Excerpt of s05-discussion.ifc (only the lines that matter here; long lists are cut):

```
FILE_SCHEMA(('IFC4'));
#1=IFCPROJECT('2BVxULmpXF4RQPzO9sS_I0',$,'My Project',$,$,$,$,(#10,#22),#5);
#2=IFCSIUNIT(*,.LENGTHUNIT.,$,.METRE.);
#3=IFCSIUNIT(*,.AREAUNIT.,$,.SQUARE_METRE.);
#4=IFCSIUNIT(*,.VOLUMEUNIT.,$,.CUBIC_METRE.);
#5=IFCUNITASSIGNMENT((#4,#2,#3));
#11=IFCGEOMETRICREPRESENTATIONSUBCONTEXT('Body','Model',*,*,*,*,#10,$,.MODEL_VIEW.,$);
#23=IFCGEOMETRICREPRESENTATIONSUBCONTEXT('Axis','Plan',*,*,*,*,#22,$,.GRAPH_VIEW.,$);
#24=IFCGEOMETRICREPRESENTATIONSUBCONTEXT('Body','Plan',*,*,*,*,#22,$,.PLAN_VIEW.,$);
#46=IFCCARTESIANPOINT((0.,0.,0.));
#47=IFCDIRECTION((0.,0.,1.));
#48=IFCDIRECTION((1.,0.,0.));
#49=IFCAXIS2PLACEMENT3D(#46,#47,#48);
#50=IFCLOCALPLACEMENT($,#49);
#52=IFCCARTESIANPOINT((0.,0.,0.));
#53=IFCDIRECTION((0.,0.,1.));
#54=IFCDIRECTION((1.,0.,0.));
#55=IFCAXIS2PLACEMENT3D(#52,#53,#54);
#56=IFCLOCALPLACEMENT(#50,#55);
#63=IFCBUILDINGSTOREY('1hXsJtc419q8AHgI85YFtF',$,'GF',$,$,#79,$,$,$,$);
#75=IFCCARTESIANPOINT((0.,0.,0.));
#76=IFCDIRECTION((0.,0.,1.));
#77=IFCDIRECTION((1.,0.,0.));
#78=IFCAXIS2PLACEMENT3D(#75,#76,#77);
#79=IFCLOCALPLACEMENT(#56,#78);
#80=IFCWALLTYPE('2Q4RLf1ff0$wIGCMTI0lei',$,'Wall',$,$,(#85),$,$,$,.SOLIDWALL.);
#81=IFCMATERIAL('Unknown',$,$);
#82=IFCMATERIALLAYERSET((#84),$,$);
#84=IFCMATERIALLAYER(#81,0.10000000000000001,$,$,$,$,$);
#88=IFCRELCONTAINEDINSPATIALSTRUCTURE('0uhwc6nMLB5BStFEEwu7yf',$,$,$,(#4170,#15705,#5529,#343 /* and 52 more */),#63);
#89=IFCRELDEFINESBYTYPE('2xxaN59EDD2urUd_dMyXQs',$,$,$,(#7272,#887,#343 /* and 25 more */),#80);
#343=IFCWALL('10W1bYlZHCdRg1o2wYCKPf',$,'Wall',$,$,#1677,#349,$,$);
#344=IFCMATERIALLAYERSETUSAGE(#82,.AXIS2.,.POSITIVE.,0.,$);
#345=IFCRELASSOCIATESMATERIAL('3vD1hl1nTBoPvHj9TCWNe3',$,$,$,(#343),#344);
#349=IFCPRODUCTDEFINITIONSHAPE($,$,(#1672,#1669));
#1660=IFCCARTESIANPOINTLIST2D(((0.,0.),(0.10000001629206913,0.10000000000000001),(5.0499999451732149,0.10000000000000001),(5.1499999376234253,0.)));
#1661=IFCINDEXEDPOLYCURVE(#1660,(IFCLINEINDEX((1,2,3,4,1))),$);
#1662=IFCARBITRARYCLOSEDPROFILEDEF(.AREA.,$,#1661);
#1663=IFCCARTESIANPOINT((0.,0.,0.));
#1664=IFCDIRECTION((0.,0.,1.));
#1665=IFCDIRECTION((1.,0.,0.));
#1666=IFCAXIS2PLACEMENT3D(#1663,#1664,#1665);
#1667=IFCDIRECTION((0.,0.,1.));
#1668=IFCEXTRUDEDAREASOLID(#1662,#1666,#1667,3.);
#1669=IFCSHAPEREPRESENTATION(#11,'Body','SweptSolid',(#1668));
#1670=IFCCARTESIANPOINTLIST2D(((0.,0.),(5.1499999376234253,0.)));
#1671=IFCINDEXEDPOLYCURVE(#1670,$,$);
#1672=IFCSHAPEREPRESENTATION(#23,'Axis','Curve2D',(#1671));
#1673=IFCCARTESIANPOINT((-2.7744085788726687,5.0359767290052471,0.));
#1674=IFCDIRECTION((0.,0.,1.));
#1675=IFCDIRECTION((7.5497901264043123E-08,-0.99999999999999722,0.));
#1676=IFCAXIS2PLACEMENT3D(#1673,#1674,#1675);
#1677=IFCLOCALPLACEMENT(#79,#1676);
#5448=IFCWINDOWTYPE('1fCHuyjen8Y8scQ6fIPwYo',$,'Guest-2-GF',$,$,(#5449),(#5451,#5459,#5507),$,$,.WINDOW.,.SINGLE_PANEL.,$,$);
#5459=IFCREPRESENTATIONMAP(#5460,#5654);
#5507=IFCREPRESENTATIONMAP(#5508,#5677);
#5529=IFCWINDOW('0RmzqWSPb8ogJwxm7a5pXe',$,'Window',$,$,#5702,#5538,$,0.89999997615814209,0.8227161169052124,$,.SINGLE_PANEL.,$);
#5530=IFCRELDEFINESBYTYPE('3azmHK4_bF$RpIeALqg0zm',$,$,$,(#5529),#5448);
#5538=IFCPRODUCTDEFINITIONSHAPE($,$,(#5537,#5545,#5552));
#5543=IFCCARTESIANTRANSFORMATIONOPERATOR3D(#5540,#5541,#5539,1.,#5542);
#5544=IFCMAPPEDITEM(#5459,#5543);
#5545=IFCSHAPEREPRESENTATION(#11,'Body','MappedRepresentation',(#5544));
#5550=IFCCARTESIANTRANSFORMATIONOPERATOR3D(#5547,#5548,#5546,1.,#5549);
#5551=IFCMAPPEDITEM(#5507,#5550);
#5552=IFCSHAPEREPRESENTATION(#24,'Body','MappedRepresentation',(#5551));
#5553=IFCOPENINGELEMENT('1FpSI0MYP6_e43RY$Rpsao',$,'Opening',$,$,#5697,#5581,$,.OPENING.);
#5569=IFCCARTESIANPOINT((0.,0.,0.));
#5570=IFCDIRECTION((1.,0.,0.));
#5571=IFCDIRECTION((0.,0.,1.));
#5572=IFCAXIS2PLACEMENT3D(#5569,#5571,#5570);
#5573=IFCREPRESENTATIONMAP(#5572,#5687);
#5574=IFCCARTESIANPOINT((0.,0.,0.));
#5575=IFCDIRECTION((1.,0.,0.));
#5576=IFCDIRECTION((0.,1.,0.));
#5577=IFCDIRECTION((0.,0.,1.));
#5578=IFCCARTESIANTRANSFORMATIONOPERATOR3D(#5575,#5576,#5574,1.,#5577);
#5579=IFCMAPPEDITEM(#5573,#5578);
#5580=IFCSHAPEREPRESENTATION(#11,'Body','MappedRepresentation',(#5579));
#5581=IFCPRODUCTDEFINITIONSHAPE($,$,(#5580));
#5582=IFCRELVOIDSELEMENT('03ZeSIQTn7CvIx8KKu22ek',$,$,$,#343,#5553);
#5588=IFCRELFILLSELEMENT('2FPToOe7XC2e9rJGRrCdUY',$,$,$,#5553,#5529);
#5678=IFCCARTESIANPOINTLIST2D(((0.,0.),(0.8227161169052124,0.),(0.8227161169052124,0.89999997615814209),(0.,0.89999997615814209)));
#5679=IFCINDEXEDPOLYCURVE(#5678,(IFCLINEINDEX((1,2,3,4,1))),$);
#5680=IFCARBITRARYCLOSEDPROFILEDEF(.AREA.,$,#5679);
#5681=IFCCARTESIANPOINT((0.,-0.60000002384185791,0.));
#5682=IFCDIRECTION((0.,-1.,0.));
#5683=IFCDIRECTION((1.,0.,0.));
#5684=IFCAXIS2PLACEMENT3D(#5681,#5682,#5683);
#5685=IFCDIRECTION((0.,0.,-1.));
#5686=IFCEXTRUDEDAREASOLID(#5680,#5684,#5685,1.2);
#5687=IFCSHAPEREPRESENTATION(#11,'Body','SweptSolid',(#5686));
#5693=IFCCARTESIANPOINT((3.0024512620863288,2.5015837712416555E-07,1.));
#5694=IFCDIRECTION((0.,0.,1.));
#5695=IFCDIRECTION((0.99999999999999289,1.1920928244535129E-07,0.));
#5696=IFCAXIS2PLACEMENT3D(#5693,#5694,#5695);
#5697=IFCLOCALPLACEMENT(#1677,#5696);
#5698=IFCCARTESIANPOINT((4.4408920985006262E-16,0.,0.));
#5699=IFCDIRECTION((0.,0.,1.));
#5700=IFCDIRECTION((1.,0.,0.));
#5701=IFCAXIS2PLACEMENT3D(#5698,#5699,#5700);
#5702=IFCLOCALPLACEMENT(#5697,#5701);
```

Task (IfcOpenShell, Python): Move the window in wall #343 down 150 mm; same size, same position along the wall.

```python
import numpy as np
import ifcopenshell
import ifcopenshell.api.geometry
import ifcopenshell.util.placement
import ifcopenshell.util.unit

model = ifcopenshell.open("s05-discussion.ifc")
unit_scale = ifcopenshell.util.unit.calculate_unit_scale(model)

window = model.by_guid("0RmzqWSPb8ogJwxm7a5pXe")
opening = window.FillsVoids[0].RelatingOpeningElement
dz = -0.15 / unit_scale

shift = np.array([0.0, 0.0, dz])
# The window is placed relative to its opening, so it follows when the opening moves.
matrix = ifcopenshell.util.placement.get_local_placement(opening.ObjectPlacement)
matrix[:3, 3] += shift
ifcopenshell.api.geometry.edit_object_placement(
    model, product=opening, matrix=matrix, is_si=False, should_transform_children=True
)

print(f"moved by {dz * unit_scale:+.3f} m")

model.write("s05-discussion_edited.ifc")
```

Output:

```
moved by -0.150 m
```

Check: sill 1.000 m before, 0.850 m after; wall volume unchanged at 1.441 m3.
